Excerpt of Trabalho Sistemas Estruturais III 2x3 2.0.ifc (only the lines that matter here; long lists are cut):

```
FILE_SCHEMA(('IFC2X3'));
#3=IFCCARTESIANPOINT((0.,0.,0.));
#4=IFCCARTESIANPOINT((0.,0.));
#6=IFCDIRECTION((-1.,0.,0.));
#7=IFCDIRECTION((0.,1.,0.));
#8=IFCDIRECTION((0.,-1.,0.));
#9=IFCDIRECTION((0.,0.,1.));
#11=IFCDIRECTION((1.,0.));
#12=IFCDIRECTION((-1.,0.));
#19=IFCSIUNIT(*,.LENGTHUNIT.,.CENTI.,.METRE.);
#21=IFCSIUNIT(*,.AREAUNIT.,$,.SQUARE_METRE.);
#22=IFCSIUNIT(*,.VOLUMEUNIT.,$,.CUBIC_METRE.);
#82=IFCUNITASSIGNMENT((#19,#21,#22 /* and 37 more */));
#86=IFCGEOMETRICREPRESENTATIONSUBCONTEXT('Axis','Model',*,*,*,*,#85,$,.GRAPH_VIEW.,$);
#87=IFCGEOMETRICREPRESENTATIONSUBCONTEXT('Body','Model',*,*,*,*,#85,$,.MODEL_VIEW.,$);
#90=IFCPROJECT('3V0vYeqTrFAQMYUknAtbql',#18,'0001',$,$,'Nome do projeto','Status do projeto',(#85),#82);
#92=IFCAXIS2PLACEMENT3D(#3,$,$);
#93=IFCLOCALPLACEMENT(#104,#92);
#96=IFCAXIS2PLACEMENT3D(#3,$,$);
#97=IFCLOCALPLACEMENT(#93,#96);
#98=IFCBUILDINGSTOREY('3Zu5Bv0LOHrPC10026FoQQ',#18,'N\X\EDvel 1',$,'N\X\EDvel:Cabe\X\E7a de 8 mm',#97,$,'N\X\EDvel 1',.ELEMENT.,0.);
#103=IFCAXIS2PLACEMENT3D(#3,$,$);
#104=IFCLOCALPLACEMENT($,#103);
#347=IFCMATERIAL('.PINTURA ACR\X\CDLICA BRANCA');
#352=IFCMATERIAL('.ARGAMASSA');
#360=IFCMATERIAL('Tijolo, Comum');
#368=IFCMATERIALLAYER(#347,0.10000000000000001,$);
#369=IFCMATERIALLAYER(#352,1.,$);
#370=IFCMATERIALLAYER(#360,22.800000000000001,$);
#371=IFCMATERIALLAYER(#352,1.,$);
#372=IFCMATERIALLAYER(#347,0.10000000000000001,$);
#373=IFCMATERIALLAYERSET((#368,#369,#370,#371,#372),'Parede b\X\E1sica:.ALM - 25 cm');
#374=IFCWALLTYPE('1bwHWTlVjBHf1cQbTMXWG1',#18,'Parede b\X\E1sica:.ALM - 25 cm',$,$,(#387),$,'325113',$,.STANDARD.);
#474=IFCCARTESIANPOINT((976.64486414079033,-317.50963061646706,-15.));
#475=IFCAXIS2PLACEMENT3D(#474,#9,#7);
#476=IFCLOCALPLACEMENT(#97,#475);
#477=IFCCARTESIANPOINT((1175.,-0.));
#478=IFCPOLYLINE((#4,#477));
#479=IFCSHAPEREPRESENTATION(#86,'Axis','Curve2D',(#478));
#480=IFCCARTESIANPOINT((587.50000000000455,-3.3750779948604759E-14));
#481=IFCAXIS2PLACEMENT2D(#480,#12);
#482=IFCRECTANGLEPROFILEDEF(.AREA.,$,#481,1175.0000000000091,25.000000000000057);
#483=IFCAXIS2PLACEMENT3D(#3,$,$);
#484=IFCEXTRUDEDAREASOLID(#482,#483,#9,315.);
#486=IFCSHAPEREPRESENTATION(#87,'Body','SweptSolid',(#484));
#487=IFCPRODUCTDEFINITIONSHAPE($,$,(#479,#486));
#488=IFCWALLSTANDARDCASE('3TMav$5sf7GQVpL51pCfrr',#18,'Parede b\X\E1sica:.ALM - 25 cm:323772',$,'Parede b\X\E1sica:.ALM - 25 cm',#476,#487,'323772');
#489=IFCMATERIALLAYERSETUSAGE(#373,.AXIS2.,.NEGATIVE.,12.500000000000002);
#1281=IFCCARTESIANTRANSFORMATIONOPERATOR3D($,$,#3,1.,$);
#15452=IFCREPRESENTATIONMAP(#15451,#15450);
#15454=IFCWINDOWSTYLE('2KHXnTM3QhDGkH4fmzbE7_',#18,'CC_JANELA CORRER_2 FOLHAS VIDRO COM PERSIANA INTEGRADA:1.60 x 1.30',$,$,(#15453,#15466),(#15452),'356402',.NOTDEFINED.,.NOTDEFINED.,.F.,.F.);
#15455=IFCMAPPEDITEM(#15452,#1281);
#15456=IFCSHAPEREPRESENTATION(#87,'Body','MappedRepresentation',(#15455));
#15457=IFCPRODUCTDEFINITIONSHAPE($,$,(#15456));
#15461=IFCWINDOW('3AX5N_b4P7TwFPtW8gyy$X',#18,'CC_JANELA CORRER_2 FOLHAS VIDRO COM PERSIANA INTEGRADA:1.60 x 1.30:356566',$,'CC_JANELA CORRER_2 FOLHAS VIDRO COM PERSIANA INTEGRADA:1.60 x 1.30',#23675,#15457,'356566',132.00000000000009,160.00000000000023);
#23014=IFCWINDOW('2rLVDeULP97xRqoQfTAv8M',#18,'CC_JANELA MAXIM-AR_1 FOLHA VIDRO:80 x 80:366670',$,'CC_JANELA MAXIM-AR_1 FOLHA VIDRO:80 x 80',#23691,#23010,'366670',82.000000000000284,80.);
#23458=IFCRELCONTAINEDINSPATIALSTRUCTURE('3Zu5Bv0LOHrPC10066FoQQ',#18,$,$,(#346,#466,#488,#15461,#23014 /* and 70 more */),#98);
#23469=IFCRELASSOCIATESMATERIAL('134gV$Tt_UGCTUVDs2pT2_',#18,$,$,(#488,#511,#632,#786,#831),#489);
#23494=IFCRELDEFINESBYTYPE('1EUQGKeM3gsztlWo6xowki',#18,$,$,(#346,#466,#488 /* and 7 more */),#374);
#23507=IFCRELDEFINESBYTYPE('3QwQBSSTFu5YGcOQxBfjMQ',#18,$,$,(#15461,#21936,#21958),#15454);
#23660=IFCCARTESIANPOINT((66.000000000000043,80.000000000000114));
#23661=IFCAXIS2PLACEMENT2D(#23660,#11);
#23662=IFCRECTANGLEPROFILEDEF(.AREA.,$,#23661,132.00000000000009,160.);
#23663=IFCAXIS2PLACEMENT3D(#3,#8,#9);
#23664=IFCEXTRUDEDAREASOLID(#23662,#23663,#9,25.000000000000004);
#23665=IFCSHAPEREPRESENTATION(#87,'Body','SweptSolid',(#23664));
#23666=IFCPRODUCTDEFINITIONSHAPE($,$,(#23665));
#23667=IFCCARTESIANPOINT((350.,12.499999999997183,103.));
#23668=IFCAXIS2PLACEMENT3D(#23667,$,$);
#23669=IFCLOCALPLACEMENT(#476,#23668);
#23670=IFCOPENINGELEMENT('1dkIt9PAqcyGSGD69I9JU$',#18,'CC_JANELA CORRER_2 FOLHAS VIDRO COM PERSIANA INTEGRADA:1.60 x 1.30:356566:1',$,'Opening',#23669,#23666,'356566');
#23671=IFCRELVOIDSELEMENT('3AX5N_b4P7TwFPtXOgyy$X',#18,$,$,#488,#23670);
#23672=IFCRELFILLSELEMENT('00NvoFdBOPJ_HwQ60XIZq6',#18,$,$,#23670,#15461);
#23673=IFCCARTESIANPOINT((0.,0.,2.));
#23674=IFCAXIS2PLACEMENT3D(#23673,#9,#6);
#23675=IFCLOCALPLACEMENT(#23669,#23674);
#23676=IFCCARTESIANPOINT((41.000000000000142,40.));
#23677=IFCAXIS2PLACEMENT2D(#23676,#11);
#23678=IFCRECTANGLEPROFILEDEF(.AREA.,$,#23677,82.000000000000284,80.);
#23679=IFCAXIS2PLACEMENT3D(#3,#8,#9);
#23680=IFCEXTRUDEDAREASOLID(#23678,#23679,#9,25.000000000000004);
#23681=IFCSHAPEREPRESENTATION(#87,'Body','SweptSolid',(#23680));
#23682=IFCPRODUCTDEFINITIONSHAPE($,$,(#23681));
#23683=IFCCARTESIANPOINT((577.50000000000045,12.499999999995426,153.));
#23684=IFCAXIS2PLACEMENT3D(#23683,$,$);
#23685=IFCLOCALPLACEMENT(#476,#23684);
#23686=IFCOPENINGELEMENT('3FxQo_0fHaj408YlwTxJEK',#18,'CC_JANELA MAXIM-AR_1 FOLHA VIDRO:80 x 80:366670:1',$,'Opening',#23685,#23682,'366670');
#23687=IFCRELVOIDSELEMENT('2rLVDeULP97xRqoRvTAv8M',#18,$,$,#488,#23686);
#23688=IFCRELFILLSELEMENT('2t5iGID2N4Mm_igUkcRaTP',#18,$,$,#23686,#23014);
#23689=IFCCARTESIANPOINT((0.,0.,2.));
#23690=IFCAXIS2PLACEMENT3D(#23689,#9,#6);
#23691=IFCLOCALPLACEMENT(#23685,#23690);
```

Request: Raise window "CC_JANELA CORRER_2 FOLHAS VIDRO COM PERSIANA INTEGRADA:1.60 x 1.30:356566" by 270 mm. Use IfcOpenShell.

```python
import numpy as np
import ifcopenshell
import ifcopenshell.api.geometry
import ifcopenshell.util.placement
import ifcopenshell.util.unit

model = ifcopenshell.open("Trabalho Sistemas Estruturais III 2x3 2.0.ifc")
unit_scale = ifcopenshell.util.unit.calculate_unit_scale(model)

window = model.by_guid("3AX5N_b4P7TwFPtW8gyy$X")
opening = window.FillsVoids[0].RelatingOpeningElement
dz = 0.27 / unit_scale

shift = np.array([0.0, 0.0, dz])
# The window is placed relative to its opening, so it follows when the opening moves.
matrix = ifcopenshell.util.placement.get_local_placement(opening.ObjectPlacement)
matrix[:3, 3] += shift
ifcopenshell.api.geometry.edit_object_placement(
    model, product=opening, matrix=matrix, is_si=False, should_transform_children=True
)

print(f"moved by {dz * unit_scale:+.3f} m")

model.write("Trabalho Sistemas Estruturais III 2x3 2.0_edited.ifc")
```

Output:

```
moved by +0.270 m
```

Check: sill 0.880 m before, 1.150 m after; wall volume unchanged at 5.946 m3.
